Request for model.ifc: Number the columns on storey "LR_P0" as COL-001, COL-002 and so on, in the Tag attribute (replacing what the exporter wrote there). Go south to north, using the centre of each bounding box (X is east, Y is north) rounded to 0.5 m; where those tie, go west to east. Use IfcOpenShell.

First a look at what the model holds.

```python
import ifcopenshell
import ifcopenshell.util.element
import ifcopenshell.util.placement

model = ifcopenshell.open("model.ifc")
print(model.schema)
storey = next(s for s in model.by_type("IfcBuildingStorey") if s.Name == "LR_P0")
columns = [e for e in ifcopenshell.util.element.get_decomposition(storey) if e.is_a("IfcColumn")]
for e in sorted(columns, key=lambda e: e.id()):
    origin = ifcopenshell.util.placement.get_local_placement(e.ObjectPlacement)[:3, 3]
    print(e.id(), e.Tag, e.Name, origin.round(2) + 0.0, sep=" | ")
```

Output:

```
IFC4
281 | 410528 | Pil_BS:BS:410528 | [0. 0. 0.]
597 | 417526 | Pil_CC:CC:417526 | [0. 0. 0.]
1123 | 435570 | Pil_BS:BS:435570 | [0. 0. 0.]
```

```python
import ifcopenshell
import ifcopenshell.geom
import ifcopenshell.util.element
import ifcopenshell.util.shape

model = ifcopenshell.open("model.ifc")
settings = ifcopenshell.geom.settings()
settings.set("use-world-coords", True)


def centre(element):
    shape = ifcopenshell.geom.create_shape(settings, element)
    return ifcopenshell.util.shape.get_bbox_centroid(shape.geometry)


storey = next(s for s in model.by_type("IfcBuildingStorey") if s.Name == "LR_P0")
columns = [e for e in ifcopenshell.util.element.get_decomposition(storey) if e.is_a("IfcColumn")]

# Insertion points can sit at a corner or the storey origin, so sort by the geometry (in metres).
centres = {e: centre(e) for e in columns}
columns.sort(key=lambda e: (round(centres[e][1] / 0.5), centres[e][0]))

for i, e in enumerate(columns, start=1):
    number = f"COL-0{i:02d}"
    e.Tag = number
    print(e.id(), number)

model.write("model_v2.ifc")
```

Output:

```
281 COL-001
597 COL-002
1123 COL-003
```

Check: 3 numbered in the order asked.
